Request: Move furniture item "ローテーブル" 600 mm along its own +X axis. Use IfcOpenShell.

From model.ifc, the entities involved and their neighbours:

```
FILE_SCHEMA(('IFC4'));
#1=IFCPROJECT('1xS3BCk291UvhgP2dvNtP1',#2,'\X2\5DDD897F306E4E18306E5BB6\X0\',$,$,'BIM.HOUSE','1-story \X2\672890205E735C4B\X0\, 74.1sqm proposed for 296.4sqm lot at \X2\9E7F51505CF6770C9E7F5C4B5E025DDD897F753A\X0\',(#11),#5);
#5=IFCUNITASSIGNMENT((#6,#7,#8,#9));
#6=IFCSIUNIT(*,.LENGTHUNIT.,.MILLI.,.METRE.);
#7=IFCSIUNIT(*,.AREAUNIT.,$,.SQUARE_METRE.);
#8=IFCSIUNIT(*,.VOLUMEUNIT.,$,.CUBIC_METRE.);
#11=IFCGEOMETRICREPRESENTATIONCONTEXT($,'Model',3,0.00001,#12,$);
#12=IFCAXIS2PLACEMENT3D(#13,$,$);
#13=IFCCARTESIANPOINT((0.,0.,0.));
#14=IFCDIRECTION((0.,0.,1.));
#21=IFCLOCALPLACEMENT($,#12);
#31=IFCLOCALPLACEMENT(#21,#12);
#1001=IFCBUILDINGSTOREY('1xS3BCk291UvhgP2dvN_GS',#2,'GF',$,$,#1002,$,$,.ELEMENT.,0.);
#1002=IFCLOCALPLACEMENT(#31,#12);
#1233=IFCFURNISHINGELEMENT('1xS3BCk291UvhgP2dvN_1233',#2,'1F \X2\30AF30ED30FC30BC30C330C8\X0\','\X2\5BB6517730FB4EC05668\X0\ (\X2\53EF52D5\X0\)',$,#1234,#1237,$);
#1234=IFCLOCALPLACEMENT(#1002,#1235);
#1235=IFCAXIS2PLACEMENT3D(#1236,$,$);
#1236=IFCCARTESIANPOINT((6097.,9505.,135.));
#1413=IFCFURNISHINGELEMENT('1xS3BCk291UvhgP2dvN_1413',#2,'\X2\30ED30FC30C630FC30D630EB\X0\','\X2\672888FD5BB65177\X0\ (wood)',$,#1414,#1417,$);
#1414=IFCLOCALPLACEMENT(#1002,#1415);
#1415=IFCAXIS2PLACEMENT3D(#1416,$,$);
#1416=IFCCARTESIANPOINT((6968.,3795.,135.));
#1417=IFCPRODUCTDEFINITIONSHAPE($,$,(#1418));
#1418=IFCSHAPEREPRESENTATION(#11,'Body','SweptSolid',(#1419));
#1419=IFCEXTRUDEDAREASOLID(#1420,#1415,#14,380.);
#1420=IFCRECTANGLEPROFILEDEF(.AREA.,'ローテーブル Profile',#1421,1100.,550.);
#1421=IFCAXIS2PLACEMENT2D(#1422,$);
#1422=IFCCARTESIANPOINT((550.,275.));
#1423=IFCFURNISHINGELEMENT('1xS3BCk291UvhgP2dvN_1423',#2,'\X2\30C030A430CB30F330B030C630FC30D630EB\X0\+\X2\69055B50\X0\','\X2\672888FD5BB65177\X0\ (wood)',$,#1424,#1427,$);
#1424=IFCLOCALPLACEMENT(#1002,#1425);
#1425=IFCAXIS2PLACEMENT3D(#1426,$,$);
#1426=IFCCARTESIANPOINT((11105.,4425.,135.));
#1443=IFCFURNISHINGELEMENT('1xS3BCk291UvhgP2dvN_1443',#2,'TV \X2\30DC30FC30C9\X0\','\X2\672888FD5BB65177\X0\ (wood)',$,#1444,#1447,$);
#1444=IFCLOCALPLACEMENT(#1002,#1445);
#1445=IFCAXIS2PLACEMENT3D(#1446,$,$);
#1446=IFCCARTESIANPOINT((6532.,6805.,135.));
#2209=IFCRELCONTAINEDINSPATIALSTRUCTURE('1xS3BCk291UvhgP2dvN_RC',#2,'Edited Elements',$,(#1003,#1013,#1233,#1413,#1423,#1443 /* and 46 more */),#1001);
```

```python
import ifcopenshell
import ifcopenshell.api.geometry
import ifcopenshell.util.placement
import ifcopenshell.util.unit

model = ifcopenshell.open("model.ifc")
unit_scale = ifcopenshell.util.unit.calculate_unit_scale(model)

item = model.by_guid("1xS3BCk291UvhgP2dvN_1413")
matrix = ifcopenshell.util.placement.get_local_placement(item.ObjectPlacement)
matrix[:3, 3] += matrix[:3, 0] * 0.6 / unit_scale
ifcopenshell.api.geometry.edit_object_placement(model, product=item, matrix=matrix, is_si=False)

print(ifcopenshell.util.placement.get_local_placement(item.ObjectPlacement).round(3) + 0.0)

model.write("model_rev.ifc")
```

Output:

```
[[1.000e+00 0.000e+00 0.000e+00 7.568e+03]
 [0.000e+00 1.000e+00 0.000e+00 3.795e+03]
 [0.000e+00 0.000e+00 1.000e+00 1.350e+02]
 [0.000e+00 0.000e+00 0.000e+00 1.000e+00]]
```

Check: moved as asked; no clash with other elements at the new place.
